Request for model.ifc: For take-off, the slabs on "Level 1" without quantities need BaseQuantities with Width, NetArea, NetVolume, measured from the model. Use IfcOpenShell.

First a look at what the model holds.

```python
import ifcopenshell
import ifcopenshell.util.element
import ifcopenshell.util.unit

model = ifcopenshell.open("model.ifc")
print(model.schema)
for unit_type in ("LENGTHUNIT", "AREAUNIT", "VOLUMEUNIT"):
    print(unit_type, ifcopenshell.util.unit.calculate_unit_scale(model, unit_type))
storey = next(s for s in model.by_type("IfcBuildingStorey") if s.Name == "Level 1")
slabs = [e for e in ifcopenshell.util.element.get_decomposition(storey) if e.is_a("IfcSlab")]
for e in sorted(slabs, key=lambda e: e.id()):
    print(e.id(), e.is_a(), e.Name, list(ifcopenshell.util.element.get_psets(e, qtos_only=True)), sep=" | ")
```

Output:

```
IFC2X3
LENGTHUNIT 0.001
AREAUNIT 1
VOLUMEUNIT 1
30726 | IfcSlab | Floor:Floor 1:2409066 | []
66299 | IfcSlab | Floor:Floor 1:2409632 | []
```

```python
import ifcopenshell
import ifcopenshell.api.pset
import ifcopenshell.geom
import ifcopenshell.util.element
import ifcopenshell.util.shape
import ifcopenshell.util.unit

model = ifcopenshell.open("model.ifc")
unit_scale = ifcopenshell.util.unit.calculate_unit_scale(model)
area_scale = ifcopenshell.util.unit.calculate_unit_scale(model, "AREAUNIT")
volume_scale = ifcopenshell.util.unit.calculate_unit_scale(model, "VOLUMEUNIT")
settings = ifcopenshell.geom.settings()

storey = next(s for s in model.by_type("IfcBuildingStorey") if s.Name == "Level 1")
slabs = [e for e in ifcopenshell.util.element.get_decomposition(storey) if e.is_a("IfcSlab")]

for e in sorted(slabs, key=lambda e: e.id()):
    if ifcopenshell.util.element.get_psets(e, qtos_only=True, should_inherit=False):
        continue
    # Geometry comes back in metres, in the element's own axes.
    shape = ifcopenshell.geom.create_shape(settings, e)
    values = {
        "Width": ifcopenshell.util.shape.get_z(shape.geometry) / unit_scale,
        "NetArea": ifcopenshell.util.shape.get_footprint_area(shape.geometry) / area_scale,
        "NetVolume": ifcopenshell.util.shape.get_volume(shape.geometry) / volume_scale,
    }
    qto = ifcopenshell.api.pset.add_qto(model, product=e, name="BaseQuantities")
    ifcopenshell.api.pset.edit_qto(model, qto=qto, properties=values)
    print(e.id(), {k: round(v, 3) for k, v in values.items()})

model.write("model_rev.ifc")
```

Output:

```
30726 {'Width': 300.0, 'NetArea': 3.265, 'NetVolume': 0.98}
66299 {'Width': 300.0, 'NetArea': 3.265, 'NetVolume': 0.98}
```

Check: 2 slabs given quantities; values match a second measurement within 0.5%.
